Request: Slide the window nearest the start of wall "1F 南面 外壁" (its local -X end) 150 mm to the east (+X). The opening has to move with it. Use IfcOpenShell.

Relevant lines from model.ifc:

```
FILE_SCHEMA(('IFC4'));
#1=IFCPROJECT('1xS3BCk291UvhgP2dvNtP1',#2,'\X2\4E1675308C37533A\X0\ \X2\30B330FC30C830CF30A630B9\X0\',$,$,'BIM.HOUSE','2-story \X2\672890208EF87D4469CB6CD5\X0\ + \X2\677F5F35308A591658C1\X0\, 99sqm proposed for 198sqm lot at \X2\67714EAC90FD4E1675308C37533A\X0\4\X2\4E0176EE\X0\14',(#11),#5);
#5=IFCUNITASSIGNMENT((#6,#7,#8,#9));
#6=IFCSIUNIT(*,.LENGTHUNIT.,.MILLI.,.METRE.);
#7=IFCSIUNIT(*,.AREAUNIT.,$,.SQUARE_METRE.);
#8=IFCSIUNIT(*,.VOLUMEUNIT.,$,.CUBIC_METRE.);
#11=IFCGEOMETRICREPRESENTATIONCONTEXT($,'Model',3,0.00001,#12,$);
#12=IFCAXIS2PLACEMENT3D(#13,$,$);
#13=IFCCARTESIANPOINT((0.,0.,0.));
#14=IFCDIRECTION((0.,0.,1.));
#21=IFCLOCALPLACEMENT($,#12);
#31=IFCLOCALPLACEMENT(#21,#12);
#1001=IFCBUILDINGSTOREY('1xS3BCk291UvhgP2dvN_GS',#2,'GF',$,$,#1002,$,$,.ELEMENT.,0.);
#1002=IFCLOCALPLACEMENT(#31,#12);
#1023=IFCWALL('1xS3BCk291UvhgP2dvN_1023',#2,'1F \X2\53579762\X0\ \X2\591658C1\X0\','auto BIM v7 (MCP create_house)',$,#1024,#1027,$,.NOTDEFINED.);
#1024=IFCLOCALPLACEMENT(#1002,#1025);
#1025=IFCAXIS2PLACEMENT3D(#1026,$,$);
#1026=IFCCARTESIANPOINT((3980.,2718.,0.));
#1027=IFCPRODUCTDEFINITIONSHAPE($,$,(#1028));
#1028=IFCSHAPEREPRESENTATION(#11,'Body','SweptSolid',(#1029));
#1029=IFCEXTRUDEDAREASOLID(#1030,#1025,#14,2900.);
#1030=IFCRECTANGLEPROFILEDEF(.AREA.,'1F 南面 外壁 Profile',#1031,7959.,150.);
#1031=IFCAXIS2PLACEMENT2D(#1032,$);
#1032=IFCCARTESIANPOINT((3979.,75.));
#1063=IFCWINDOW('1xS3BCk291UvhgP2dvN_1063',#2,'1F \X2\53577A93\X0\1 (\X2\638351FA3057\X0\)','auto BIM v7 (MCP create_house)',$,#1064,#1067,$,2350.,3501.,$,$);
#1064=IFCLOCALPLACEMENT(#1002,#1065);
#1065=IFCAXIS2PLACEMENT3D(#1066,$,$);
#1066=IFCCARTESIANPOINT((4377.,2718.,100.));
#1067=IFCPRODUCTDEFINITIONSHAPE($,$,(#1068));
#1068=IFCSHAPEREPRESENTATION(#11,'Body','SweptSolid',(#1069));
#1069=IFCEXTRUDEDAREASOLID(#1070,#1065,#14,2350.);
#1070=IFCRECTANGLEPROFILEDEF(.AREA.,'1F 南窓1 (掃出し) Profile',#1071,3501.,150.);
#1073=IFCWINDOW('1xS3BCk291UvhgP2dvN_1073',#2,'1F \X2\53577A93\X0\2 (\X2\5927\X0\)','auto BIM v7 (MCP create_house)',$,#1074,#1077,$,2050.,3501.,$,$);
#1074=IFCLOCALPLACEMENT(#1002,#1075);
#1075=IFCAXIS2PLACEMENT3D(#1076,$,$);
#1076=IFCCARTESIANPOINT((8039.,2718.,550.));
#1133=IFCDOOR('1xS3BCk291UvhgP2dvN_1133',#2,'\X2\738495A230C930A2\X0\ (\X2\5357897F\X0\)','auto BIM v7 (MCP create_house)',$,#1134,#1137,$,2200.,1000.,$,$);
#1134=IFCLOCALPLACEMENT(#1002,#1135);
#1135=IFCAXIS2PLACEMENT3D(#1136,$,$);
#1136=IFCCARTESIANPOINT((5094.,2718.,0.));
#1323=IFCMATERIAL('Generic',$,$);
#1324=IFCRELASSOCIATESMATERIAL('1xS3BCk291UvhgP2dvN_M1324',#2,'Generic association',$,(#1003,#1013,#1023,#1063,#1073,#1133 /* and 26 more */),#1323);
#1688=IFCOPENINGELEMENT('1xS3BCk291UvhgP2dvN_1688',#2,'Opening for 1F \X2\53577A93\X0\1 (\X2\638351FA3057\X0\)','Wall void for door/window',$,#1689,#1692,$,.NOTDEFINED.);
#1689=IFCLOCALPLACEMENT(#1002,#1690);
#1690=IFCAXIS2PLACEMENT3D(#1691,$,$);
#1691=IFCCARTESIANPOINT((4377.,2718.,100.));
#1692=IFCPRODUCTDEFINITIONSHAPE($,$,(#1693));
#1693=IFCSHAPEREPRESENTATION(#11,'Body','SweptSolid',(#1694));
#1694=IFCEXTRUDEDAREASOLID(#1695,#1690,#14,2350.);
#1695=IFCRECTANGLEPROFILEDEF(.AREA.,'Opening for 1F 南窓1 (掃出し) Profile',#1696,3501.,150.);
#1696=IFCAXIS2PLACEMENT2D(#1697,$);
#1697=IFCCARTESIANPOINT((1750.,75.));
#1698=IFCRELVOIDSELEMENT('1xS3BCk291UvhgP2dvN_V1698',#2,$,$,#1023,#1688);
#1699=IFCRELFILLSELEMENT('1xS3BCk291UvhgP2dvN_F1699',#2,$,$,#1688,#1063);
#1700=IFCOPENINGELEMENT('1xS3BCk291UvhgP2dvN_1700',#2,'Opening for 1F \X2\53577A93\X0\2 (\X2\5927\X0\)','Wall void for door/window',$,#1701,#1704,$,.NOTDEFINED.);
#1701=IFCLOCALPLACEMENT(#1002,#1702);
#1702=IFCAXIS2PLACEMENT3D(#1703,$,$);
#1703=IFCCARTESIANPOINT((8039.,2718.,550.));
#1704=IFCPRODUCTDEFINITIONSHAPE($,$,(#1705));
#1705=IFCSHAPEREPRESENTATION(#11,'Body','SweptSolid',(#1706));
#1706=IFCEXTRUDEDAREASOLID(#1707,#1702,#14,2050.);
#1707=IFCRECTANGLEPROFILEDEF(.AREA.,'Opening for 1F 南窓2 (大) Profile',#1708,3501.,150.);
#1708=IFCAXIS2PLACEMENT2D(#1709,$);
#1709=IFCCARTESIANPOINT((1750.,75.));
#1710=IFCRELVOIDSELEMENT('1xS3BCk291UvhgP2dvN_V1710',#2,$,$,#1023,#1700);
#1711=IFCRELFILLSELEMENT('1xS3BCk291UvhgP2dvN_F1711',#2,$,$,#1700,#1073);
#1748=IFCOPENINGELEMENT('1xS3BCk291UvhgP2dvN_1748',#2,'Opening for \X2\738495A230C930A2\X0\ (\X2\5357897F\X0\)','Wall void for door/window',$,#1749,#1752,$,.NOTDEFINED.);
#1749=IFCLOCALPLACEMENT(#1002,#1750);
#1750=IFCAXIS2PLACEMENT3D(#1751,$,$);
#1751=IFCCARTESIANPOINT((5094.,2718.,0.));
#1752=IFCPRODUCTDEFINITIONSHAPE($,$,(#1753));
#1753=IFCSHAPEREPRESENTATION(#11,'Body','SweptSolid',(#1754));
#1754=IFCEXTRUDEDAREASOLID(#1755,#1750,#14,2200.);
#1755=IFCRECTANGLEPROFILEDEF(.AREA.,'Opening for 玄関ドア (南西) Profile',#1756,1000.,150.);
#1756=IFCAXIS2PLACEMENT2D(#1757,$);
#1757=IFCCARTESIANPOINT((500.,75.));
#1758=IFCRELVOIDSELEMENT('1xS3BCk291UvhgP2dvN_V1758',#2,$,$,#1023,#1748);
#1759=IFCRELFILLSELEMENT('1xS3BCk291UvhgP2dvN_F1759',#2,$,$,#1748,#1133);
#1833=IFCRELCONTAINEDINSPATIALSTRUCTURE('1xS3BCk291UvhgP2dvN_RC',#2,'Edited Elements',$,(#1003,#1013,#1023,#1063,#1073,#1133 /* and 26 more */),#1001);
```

```python
import ifcopenshell
import ifcopenshell.api.geometry
import ifcopenshell.util.placement
import ifcopenshell.util.unit

model = ifcopenshell.open("model.ifc")
unit_scale = ifcopenshell.util.unit.calculate_unit_scale(model)

window = model.by_guid("1xS3BCk291UvhgP2dvN_1063")
opening = window.FillsVoids[0].RelatingOpeningElement
wall = opening.VoidsElements[0].RelatingBuildingElement

wall_matrix = ifcopenshell.util.placement.get_local_placement(wall.ObjectPlacement)
shift = wall_matrix[:3, 0] * 0.15 / unit_scale
before = ifcopenshell.util.placement.get_local_placement(window.ObjectPlacement)[:3, 3].copy()

# The window is not placed relative to its opening, so move both.
for product in (opening, window):
    matrix = ifcopenshell.util.placement.get_local_placement(product.ObjectPlacement)
    matrix[:3, 3] += shift
    ifcopenshell.api.geometry.edit_object_placement(model, product=product, matrix=matrix, is_si=False)

after = ifcopenshell.util.placement.get_local_placement(window.ObjectPlacement)[:3, 3]
print("window moved by", (after - before).round(3) + 0.0)

model.write("model-out.ifc")
```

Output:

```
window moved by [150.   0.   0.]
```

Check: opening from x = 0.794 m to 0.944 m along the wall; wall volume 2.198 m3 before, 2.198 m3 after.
